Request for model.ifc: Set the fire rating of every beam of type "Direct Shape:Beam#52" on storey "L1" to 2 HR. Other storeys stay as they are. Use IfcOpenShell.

First a look at what the model holds.

```python
import ifcopenshell
import ifcopenshell.util.element

model = ifcopenshell.open("model.ifc")
print(model.schema)
storey = next(s for s in model.by_type("IfcBuildingStorey") if s.Name == "L1")
beams = [e for e in ifcopenshell.util.element.get_decomposition(storey) if e.is_a("IfcBeam")]
seen = {}
for e in beams:
    element_type = ifcopenshell.util.element.get_type(e)
    key = (element_type.Name if element_type != e and element_type else None, ifcopenshell.util.element.get_pset(e, "Pset_BeamCommon", "FireRating"))
    seen[key] = seen.get(key, 0) + 1
for (name, value), count in sorted(seen.items(), key=str):
    print(count, "x", name, "|", value)
```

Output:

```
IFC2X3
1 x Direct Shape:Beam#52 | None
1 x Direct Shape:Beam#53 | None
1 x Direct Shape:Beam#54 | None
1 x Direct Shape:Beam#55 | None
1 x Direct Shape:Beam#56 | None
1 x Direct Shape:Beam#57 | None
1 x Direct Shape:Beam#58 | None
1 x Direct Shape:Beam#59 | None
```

```python
import ifcopenshell
import ifcopenshell.api.pset
import ifcopenshell.util.element

model = ifcopenshell.open("model.ifc")

storey = next(s for s in model.by_type("IfcBuildingStorey") if s.Name == "L1")
beams = [e for e in ifcopenshell.util.element.get_decomposition(storey) if e.is_a("IfcBeam")]

count = 0
for e in beams:
    element_type = ifcopenshell.util.element.get_type(e)
    if element_type in (None, e) or element_type.Name != "Direct Shape:Beam#52":
        continue
    # add_pset returns the element's existing set when there is one.
    pset = ifcopenshell.api.pset.add_pset(model, product=e, name="Pset_BeamCommon")
    ifcopenshell.api.pset.edit_pset(model, pset=pset, properties={"FireRating": "2 HR"})
    count += 1

print(count, "beams updated")

model.write("model_updated.ifc")
```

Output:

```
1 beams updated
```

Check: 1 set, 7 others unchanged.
